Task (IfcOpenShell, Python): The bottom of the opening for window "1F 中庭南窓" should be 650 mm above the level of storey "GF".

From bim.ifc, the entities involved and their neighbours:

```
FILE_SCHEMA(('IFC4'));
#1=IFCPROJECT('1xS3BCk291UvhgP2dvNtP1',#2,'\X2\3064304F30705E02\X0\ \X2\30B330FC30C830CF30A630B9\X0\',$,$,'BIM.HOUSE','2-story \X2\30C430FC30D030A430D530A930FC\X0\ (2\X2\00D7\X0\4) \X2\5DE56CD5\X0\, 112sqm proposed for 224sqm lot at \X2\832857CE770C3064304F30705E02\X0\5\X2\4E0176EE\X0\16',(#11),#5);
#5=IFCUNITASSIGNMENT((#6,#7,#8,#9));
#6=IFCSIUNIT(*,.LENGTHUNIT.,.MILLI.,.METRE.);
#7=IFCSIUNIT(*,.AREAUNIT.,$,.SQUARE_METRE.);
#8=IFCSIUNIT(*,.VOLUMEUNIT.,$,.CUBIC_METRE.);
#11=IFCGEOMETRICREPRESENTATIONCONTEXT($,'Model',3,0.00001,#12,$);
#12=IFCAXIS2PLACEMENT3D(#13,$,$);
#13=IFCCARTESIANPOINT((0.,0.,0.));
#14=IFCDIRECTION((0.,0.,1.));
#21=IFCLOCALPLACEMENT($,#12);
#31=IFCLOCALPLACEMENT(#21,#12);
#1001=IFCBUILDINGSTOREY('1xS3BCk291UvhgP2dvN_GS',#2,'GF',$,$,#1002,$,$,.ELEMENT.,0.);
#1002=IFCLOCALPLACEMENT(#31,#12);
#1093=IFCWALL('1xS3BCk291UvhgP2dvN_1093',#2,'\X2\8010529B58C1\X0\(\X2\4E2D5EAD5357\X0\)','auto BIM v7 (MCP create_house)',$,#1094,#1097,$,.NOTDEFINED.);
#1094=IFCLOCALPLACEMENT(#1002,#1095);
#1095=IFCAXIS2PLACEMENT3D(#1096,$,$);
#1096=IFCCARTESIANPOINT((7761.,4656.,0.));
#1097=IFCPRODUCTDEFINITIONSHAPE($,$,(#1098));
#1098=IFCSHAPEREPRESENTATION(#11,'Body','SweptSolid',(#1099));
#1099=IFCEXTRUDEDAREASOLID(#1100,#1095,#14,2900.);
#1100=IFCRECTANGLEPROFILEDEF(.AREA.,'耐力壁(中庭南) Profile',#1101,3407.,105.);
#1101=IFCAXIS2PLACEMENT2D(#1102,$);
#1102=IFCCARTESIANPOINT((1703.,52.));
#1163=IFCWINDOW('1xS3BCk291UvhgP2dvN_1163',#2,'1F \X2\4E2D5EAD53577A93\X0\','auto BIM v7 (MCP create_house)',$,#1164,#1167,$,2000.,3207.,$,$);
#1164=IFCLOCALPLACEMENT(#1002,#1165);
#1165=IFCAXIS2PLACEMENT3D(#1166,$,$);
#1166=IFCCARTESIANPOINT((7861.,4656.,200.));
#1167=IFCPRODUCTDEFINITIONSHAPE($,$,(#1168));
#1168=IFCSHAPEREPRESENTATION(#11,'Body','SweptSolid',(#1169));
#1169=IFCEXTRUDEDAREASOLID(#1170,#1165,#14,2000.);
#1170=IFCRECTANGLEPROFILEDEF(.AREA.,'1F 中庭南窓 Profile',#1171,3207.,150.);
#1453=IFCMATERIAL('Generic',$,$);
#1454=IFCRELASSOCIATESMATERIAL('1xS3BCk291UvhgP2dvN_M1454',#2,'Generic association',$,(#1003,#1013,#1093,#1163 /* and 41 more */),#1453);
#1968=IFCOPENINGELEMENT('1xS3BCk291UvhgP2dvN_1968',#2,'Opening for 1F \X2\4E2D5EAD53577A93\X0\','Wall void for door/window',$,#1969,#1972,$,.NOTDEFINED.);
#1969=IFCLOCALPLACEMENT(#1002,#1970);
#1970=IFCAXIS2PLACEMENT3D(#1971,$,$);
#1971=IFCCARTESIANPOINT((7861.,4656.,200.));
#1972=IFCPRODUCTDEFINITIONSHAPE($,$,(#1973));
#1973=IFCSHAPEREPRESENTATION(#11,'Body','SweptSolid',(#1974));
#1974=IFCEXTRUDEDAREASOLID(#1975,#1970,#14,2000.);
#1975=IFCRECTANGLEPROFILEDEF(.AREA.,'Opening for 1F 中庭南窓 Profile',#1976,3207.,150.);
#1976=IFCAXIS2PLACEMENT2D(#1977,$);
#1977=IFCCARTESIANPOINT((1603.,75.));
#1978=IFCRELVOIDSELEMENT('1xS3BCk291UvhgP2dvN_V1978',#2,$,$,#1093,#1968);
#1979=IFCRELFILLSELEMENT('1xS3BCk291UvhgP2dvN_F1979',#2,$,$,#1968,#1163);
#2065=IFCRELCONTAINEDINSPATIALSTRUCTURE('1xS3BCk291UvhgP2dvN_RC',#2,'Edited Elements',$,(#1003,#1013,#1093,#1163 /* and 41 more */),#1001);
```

```python
import numpy as np
import ifcopenshell
import ifcopenshell.api.geometry
import ifcopenshell.geom
import ifcopenshell.util.element
import ifcopenshell.util.placement
import ifcopenshell.util.shape
import ifcopenshell.util.unit

model = ifcopenshell.open("bim.ifc")
unit_scale = ifcopenshell.util.unit.calculate_unit_scale(model)

window = model.by_guid("1xS3BCk291UvhgP2dvN_1163")
opening = window.FillsVoids[0].RelatingOpeningElement
storey = ifcopenshell.util.element.get_container(window, ifc_class="IfcBuildingStorey")
level = ifcopenshell.util.placement.get_local_placement(storey.ObjectPlacement)[2, 3]

# The opening's origin need not be at the sill, so measure its lowest point.
shape = ifcopenshell.geom.create_shape(ifcopenshell.geom.settings(), opening)
bottom = ifcopenshell.util.shape.get_shape_bottom_elevation(shape, shape.geometry) / unit_scale
dz = level + 0.65 / unit_scale - bottom

shift = np.array([0.0, 0.0, dz])
# The window is not placed relative to its opening, so move both.
for product in (opening, window):
    matrix = ifcopenshell.util.placement.get_local_placement(product.ObjectPlacement)
    matrix[:3, 3] += shift
    ifcopenshell.api.geometry.edit_object_placement(model, product=product, matrix=matrix, is_si=False)

print(f"moved by {dz * unit_scale:+.3f} m")

model.write("bim-out.ifc")
```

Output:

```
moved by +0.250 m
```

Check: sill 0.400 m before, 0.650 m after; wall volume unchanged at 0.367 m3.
